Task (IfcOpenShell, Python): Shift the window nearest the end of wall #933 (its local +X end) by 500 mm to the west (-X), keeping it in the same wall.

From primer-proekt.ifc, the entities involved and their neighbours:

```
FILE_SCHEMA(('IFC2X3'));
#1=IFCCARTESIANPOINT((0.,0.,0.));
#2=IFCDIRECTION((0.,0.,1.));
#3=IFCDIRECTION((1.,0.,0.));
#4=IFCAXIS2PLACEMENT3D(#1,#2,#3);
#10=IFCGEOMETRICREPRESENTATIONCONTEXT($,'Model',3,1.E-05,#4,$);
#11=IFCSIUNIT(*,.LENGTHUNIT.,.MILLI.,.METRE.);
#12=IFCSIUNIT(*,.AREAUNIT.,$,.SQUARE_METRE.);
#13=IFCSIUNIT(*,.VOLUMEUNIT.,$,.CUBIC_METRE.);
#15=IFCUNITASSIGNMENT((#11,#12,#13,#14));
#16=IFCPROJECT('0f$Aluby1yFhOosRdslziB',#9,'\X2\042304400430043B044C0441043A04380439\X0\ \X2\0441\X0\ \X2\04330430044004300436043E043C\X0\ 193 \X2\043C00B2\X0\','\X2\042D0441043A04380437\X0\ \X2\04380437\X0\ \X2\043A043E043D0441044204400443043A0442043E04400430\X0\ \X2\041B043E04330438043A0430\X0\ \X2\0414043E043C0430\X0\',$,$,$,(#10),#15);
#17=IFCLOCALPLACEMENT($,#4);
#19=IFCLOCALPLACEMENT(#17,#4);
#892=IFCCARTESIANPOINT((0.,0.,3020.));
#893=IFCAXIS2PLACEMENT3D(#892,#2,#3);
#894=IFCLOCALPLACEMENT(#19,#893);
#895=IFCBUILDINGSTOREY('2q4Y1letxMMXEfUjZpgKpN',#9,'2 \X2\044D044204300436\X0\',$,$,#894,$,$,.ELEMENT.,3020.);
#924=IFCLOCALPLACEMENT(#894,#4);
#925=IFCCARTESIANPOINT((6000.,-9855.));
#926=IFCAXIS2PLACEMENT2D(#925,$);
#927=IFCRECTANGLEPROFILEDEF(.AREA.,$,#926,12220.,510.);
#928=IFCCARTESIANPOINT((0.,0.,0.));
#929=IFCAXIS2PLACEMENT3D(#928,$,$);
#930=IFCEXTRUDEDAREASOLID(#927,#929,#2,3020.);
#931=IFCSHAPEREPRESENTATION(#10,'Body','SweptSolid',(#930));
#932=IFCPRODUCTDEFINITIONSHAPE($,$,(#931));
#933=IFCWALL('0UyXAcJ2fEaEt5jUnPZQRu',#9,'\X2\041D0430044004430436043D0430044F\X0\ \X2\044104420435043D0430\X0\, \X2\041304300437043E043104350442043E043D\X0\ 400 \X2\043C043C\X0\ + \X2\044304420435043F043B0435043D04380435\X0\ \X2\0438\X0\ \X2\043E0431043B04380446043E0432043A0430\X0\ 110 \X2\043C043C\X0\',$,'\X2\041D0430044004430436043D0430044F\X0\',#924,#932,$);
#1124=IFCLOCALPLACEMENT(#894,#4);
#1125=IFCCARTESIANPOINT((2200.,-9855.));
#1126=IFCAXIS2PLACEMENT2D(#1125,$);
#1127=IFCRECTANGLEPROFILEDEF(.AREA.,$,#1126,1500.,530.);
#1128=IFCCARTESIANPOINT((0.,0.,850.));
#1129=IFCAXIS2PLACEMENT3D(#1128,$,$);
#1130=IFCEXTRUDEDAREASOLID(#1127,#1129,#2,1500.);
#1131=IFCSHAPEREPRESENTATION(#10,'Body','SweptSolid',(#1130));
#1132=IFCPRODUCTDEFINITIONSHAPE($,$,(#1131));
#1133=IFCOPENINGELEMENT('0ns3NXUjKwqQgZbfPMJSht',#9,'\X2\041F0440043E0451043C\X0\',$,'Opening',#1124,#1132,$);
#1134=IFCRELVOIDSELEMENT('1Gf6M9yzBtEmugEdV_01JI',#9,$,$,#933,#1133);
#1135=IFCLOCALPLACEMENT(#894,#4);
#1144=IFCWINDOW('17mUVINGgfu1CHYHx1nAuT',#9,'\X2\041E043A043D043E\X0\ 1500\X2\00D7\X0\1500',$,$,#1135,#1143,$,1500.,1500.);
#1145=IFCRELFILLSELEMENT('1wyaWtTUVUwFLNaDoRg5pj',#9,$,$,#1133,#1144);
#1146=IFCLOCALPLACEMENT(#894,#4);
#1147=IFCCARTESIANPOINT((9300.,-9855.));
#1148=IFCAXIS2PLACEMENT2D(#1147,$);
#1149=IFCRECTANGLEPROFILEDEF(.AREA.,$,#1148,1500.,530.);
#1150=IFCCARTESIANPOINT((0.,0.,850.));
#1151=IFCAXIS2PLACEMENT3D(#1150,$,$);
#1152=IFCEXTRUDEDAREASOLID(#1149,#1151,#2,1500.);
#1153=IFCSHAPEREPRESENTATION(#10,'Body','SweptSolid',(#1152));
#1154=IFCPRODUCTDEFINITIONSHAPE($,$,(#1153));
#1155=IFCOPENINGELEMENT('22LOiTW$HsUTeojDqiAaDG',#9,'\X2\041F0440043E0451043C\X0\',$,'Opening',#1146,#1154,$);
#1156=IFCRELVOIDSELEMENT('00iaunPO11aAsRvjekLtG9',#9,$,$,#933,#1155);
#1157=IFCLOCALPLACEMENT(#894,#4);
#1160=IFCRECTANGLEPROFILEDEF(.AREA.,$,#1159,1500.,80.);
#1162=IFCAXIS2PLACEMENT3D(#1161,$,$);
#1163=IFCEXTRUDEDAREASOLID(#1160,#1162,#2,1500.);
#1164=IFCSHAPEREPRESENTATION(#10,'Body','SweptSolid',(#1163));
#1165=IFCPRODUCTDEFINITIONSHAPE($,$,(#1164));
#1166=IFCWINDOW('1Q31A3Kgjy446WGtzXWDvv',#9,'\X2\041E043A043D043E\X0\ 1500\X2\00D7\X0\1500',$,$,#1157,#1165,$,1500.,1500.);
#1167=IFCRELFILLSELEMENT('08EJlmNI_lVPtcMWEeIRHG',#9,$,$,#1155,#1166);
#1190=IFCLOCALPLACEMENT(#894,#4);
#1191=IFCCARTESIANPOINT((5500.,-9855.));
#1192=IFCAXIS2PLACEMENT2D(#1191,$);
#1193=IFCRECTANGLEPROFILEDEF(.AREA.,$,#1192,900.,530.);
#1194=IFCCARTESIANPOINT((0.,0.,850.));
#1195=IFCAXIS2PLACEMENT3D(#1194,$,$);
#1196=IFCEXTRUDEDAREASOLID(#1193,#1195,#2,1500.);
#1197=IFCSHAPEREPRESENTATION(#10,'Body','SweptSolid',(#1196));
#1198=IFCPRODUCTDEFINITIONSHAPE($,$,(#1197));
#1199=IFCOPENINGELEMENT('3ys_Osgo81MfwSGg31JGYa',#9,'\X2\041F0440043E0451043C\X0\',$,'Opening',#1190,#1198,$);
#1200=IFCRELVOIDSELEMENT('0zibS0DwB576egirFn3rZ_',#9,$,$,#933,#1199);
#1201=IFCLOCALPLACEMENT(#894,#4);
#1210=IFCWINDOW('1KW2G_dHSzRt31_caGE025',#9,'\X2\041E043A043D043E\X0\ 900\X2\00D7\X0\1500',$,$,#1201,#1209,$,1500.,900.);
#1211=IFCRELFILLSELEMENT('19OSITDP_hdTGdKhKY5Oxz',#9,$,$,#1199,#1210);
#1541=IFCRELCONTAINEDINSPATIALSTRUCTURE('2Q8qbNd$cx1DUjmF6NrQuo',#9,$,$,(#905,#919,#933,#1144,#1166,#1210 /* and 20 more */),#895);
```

```python
import ifcopenshell
import ifcopenshell.api.geometry
import ifcopenshell.util.placement

model = ifcopenshell.open("primer-proekt.ifc")

window = model.by_guid("1Q31A3Kgjy446WGtzXWDvv")
opening = window.FillsVoids[0].RelatingOpeningElement
wall = opening.VoidsElements[0].RelatingBuildingElement

wall_matrix = ifcopenshell.util.placement.get_local_placement(wall.ObjectPlacement)
shift = wall_matrix[:3, 0] * -500.0
before = ifcopenshell.util.placement.get_local_placement(window.ObjectPlacement)[:3, 3].copy()

# The window is not placed relative to its opening, so move both.
for product in (opening, window):
    matrix = ifcopenshell.util.placement.get_local_placement(product.ObjectPlacement)
    matrix[:3, 3] += shift
    ifcopenshell.api.geometry.edit_object_placement(model, product=product, matrix=matrix, is_si=False)

after = ifcopenshell.util.placement.get_local_placement(window.ObjectPlacement)[:3, 3]
print("window moved by", (after - before).round(3) + 0.0)

model.write("primer-proekt-out.ifc")
```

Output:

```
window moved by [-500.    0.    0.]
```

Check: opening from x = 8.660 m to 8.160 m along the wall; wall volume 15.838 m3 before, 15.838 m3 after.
